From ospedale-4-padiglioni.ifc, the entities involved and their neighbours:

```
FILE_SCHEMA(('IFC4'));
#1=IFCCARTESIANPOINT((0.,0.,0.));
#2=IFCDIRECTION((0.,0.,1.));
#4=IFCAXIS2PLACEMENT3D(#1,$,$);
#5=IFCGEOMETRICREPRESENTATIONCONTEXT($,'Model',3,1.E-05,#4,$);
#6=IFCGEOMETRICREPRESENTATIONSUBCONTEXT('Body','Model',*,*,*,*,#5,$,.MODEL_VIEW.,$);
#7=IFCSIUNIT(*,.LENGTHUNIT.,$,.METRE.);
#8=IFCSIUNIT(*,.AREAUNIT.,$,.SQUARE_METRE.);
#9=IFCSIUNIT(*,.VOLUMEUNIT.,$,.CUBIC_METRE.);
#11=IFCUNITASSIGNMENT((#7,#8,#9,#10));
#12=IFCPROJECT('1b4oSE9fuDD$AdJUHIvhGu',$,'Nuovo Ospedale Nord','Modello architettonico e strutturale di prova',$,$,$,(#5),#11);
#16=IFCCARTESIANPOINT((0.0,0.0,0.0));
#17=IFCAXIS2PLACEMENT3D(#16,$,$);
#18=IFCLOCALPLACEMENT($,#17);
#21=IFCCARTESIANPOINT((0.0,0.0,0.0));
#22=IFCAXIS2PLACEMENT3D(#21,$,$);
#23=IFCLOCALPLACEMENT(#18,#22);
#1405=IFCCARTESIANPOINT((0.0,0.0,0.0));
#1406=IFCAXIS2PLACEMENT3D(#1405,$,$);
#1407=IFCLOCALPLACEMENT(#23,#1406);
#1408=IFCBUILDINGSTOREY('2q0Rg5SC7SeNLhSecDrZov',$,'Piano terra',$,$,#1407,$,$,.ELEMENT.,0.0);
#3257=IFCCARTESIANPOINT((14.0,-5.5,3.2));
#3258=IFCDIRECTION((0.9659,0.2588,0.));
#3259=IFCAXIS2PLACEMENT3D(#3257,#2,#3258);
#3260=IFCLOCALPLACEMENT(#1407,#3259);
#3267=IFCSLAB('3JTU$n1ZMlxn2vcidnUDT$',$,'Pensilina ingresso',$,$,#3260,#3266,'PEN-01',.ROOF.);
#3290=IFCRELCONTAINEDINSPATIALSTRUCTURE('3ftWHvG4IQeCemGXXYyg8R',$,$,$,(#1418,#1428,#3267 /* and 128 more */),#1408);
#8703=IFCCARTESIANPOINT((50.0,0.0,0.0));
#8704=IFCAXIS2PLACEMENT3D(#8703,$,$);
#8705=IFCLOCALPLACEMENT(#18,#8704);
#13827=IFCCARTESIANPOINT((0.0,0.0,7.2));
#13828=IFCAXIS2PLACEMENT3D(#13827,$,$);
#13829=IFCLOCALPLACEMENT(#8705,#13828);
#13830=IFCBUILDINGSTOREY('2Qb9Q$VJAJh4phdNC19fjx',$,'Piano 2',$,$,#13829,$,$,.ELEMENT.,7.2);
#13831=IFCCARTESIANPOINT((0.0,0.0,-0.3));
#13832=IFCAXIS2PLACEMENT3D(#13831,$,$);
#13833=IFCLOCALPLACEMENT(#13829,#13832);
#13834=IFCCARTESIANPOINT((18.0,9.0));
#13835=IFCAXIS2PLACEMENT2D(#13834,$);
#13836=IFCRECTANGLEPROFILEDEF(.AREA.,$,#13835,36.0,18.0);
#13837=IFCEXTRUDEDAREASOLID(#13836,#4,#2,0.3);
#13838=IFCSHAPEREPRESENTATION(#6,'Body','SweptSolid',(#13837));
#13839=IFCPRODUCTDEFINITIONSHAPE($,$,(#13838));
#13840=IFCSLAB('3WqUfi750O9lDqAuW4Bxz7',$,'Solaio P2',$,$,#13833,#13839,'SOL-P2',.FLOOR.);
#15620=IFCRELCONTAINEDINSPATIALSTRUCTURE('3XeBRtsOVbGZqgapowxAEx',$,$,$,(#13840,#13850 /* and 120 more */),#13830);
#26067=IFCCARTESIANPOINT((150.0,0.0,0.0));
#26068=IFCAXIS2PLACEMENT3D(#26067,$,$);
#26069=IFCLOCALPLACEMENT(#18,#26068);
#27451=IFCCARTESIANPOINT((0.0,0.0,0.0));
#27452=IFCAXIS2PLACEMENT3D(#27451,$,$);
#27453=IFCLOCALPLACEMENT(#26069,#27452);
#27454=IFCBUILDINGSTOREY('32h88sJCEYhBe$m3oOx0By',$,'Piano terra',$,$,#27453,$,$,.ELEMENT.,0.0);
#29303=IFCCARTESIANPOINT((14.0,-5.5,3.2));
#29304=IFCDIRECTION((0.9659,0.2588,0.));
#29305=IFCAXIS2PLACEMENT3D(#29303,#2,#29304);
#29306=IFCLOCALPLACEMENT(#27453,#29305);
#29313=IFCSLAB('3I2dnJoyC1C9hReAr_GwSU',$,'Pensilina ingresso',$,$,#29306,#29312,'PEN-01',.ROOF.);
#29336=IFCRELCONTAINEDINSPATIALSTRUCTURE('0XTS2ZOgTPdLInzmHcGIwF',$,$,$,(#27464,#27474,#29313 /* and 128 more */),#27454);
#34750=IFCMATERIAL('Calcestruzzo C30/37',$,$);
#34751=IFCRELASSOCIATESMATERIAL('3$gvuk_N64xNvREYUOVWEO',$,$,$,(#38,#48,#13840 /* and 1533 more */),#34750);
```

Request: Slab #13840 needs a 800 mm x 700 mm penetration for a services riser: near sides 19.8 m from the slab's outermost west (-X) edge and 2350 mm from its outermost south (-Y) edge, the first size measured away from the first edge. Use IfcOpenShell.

```python
import numpy as np
import ifcopenshell
import ifcopenshell.api.feature
import ifcopenshell.api.geometry
import ifcopenshell.api.root
import ifcopenshell.geom
import ifcopenshell.util.placement
import ifcopenshell.util.representation
import ifcopenshell.util.shape
import ifcopenshell.util.unit

model = ifcopenshell.open("ospedale-4-padiglioni.ifc")
unit_scale = ifcopenshell.util.unit.calculate_unit_scale(model)
settings = ifcopenshell.geom.settings()


def volume(element):
    """Net volume in cubic metres, openings subtracted."""
    shape = ifcopenshell.geom.create_shape(settings, element)
    return ifcopenshell.util.shape.get_volume(shape.geometry)


slab = model.by_guid("3WqUfi750O9lDqAuW4Bxz7")
before = volume(slab)

# Extent in the slab's own axes, in metres. The edges named are its -X and -Y sides.
slab_shape = ifcopenshell.geom.create_shape(settings, slab)
vertices = ifcopenshell.util.shape.get_vertices(slab_shape.geometry)
x_min, y_min, bottom = vertices.min(axis=0)
top = vertices[:, 2].max()

opening = ifcopenshell.api.root.create_entity(model, ifc_class="IfcOpeningElement", name="Services riser opening", predefined_type="OPENING")
context = ifcopenshell.util.representation.get_context(model, "Model", "Body", "MODEL_VIEW")
width, depth = 0.8, 0.7
outline = [(0.0, 0.0), (width, 0.0), (width, depth), (0.0, depth), (0.0, 0.0)]
# Overshoot both faces by 50 mm so the cut is clean.
shape = ifcopenshell.api.geometry.add_slab_representation(
    model, context=context, depth=top - bottom + 0.1, polyline=outline
)
ifcopenshell.api.geometry.assign_representation(model, product=opening, representation=shape)

matrix = ifcopenshell.util.placement.get_local_placement(slab.ObjectPlacement)
matrix[:, 3] = matrix @ np.append(np.array([x_min + 19.8, y_min + 2.35, bottom - 0.05]) / unit_scale, 1.0)
ifcopenshell.api.geometry.edit_object_placement(model, product=opening, matrix=matrix, is_si=False)
ifcopenshell.api.feature.add_feature(model, feature=opening, element=slab)

after = volume(slab)

print(f"slab volume {before:.3f} -> {after:.3f} m3")

model.write("ospedale-4-padiglioni_rev.ifc")
```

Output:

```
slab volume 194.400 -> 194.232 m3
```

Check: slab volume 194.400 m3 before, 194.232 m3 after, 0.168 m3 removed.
